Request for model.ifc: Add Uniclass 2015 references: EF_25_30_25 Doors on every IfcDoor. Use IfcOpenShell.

First a look at what the model holds.

```python
import ifcopenshell

model = ifcopenshell.open("model.ifc")
print(model.schema)
print("classifications:", [c.Name for c in model.by_type("IfcClassification")])
for ifc_class in ("IfcDoor", "IfcRoof", "IfcStair", "IfcWall", "IfcWindow"):
    print(ifc_class, len(model.by_type(ifc_class)))
```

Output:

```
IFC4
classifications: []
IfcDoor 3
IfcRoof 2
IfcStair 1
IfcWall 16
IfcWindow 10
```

```python
import ifcopenshell
import ifcopenshell.api.classification

model = ifcopenshell.open("model.ifc")

system = ifcopenshell.api.classification.add_classification(model, classification="Uniclass 2015")

codes = {
    "IfcDoor": ("EF_25_30_25", "Doors"),
}
for ifc_class, (code, name) in codes.items():
    products = model.by_type(ifc_class)
    ifcopenshell.api.classification.add_reference(
        model, products=products, classification=system, identification=code, name=name
    )
    print(code, len(products))

model.write("model_updated.ifc")
```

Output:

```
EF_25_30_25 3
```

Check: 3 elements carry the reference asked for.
